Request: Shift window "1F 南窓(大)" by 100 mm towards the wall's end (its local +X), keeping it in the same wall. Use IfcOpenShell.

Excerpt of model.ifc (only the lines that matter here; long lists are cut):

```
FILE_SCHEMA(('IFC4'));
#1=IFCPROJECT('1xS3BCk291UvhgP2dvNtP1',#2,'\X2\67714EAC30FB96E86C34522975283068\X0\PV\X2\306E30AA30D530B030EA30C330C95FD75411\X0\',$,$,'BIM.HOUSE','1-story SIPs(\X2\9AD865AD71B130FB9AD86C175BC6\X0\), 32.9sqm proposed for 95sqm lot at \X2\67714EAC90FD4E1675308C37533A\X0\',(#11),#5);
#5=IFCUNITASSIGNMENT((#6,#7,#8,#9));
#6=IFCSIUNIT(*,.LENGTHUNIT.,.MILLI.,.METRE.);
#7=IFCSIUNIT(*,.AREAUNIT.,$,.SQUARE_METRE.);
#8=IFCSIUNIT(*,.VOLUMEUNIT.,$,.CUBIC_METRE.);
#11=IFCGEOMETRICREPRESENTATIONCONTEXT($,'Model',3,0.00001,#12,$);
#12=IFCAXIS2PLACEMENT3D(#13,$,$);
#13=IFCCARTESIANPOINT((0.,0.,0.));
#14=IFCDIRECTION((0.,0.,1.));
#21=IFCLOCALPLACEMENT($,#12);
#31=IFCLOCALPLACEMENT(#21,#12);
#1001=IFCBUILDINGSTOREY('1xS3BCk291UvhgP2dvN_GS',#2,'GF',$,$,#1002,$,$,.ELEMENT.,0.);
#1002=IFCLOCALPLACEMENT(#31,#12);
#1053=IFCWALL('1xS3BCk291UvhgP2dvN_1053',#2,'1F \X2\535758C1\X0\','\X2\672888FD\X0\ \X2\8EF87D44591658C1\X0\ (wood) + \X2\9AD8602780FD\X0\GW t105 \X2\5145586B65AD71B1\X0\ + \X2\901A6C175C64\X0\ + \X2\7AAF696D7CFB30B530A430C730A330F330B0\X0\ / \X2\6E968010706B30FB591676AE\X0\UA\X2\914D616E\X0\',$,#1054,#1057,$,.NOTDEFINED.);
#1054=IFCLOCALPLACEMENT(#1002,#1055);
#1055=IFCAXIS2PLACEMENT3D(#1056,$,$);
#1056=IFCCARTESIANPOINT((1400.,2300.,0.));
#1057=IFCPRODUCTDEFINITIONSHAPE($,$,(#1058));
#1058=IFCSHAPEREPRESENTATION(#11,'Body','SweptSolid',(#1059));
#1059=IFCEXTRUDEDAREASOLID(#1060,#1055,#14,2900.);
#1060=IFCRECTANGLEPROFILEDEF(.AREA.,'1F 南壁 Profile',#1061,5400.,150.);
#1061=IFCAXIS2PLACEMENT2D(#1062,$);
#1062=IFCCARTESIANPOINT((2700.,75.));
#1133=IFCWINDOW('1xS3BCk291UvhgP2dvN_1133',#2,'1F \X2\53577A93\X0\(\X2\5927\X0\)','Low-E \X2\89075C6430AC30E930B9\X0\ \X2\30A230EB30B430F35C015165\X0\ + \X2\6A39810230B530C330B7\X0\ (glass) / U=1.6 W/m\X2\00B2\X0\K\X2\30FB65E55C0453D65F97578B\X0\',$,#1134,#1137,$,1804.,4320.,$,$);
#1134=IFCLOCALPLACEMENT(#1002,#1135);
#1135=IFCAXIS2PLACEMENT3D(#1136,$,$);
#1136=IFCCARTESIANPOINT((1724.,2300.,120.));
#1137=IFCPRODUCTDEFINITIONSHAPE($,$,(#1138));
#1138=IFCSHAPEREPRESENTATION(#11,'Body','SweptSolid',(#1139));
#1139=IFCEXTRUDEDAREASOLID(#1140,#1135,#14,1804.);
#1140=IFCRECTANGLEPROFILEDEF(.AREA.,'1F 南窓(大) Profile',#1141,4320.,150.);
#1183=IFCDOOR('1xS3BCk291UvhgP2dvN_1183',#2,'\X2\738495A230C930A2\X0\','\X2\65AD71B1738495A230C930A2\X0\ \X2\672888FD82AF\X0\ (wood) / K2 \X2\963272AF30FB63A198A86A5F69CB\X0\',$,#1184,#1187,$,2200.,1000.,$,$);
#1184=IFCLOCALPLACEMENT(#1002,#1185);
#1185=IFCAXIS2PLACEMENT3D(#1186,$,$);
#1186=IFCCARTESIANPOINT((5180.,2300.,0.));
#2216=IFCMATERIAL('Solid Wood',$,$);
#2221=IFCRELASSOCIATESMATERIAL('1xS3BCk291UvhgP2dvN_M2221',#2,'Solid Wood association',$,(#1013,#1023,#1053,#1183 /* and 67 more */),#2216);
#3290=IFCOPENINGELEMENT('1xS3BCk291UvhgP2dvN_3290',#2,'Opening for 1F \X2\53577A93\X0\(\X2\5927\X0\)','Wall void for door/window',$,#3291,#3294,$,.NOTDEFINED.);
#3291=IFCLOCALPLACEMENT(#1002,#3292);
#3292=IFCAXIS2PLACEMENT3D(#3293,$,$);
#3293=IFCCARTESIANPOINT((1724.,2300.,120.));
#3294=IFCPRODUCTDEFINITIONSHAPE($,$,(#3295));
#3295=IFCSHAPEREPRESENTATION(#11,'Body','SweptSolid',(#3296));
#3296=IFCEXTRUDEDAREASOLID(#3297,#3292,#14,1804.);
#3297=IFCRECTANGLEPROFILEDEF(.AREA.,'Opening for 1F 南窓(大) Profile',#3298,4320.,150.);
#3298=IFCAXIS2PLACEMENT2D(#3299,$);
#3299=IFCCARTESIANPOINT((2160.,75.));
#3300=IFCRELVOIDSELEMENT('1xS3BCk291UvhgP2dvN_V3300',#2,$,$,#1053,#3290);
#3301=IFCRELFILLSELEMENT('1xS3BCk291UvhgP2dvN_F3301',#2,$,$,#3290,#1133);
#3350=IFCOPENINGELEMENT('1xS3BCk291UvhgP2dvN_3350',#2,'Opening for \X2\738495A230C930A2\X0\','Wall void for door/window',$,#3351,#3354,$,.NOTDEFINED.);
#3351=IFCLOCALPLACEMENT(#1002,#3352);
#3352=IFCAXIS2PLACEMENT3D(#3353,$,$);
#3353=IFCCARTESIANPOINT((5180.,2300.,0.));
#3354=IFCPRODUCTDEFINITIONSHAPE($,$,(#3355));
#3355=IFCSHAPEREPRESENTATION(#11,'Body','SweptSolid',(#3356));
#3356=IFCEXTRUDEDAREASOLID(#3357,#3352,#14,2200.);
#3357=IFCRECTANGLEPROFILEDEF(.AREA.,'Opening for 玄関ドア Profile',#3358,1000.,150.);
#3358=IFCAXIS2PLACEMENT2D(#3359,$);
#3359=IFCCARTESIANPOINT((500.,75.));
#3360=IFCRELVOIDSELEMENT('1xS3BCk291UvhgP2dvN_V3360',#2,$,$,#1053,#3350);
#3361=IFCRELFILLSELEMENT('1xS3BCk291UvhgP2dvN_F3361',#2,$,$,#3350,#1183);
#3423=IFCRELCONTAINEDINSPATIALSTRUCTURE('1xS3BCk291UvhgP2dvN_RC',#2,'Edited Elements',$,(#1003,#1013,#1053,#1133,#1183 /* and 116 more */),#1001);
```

```python
import ifcopenshell
import ifcopenshell.api.geometry
import ifcopenshell.util.placement
import ifcopenshell.util.unit

model = ifcopenshell.open("model.ifc")
unit_scale = ifcopenshell.util.unit.calculate_unit_scale(model)

window = model.by_guid("1xS3BCk291UvhgP2dvN_1133")
opening = window.FillsVoids[0].RelatingOpeningElement
wall = opening.VoidsElements[0].RelatingBuildingElement

wall_matrix = ifcopenshell.util.placement.get_local_placement(wall.ObjectPlacement)
shift = wall_matrix[:3, 0] * 0.1 / unit_scale
before = ifcopenshell.util.placement.get_local_placement(window.ObjectPlacement)[:3, 3].copy()

# The window is not placed relative to its opening, so move both.
for product in (opening, window):
    matrix = ifcopenshell.util.placement.get_local_placement(product.ObjectPlacement)
    matrix[:3, 3] += shift
    ifcopenshell.api.geometry.edit_object_placement(model, product=product, matrix=matrix, is_si=False)

after = ifcopenshell.util.placement.get_local_placement(window.ObjectPlacement)[:3, 3]
print("window moved by", (after - before).round(3) + 0.0)

model.write("model_rev.ifc")
```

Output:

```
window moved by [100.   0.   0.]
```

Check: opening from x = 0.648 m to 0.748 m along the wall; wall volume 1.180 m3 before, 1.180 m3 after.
